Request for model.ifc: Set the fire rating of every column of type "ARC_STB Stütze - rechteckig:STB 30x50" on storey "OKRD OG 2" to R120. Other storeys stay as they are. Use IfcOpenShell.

First a look at what the model holds.

```python
import ifcopenshell
import ifcopenshell.util.element

model = ifcopenshell.open("model.ifc")
print(model.schema)
storey = next(s for s in model.by_type("IfcBuildingStorey") if s.Name == "OKRD OG 2")
columns = [e for e in ifcopenshell.util.element.get_decomposition(storey) if e.is_a("IfcColumn")]
seen = {}
for e in columns:
    element_type = ifcopenshell.util.element.get_type(e)
    key = (element_type.Name if element_type != e and element_type else None, ifcopenshell.util.element.get_pset(e, "Pset_ColumnCommon", "FireRating"))
    seen[key] = seen.get(key, 0) + 1
for (name, value), count in sorted(seen.items(), key=str):
    print(count, "x", name, "|", value)
```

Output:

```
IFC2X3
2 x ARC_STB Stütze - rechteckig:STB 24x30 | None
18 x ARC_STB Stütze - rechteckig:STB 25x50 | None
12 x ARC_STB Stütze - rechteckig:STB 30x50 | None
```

```python
import ifcopenshell
import ifcopenshell.api.pset
import ifcopenshell.util.element

model = ifcopenshell.open("model.ifc")

storey = next(s for s in model.by_type("IfcBuildingStorey") if s.Name == "OKRD OG 2")
columns = [e for e in ifcopenshell.util.element.get_decomposition(storey) if e.is_a("IfcColumn")]

count = 0
for e in columns:
    element_type = ifcopenshell.util.element.get_type(e)
    if element_type in (None, e) or element_type.Name != "ARC_STB Stütze - rechteckig:STB 30x50":
        continue
    found = ifcopenshell.util.element.get_pset(e, "Pset_ColumnCommon", should_inherit=False)
    if found:
        pset = model.by_id(found["id"])
        if len(ifcopenshell.util.element.get_elements_by_pset(pset)) > 1:
            pset = ifcopenshell.api.pset.unshare_pset(model, products=[e], pset=pset)[0]
    else:
        pset = ifcopenshell.api.pset.add_pset(model, product=e, name="Pset_ColumnCommon")
    ifcopenshell.api.pset.edit_pset(model, pset=pset, properties={"FireRating": "R120"})
    count += 1

print(count, "columns updated")

model.write("model-out.ifc")
```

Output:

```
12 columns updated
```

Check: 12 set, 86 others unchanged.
